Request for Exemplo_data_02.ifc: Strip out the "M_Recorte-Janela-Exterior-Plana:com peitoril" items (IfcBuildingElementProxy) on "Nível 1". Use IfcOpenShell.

First a look at what the model holds.

```python
import ifcopenshell
import ifcopenshell.util.element

model = ifcopenshell.open("Exemplo_data_02.ifc")
print(model.schema)
storey = next(s for s in model.by_type("IfcBuildingStorey") if s.Name == "Nível 1")
proxies = [e for e in ifcopenshell.util.element.get_decomposition(storey) if e.is_a("IfcBuildingElementProxy")]
seen = {}
for e in proxies:
    element_type = ifcopenshell.util.element.get_type(e)
    name = element_type.Name if element_type not in (None, e) else None
    seen[name] = seen.get(name, 0) + 1
for name, count in sorted(seen.items(), key=str):
    print(count, "x", name)
```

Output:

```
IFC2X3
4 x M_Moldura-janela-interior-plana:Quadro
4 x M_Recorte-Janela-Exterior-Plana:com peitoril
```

```python
import ifcopenshell
import ifcopenshell.api.root
import ifcopenshell.util.element

model = ifcopenshell.open("Exemplo_data_02.ifc")

storey = next(s for s in model.by_type("IfcBuildingStorey") if s.Name == "Nível 1")
proxies = [e for e in ifcopenshell.util.element.get_decomposition(storey) if e.is_a("IfcBuildingElementProxy")]
targets = [e for e in proxies if (t := ifcopenshell.util.element.get_type(e)) not in (None, e) and t.Name == "M_Recorte-Janela-Exterior-Plana:com peitoril"]

for e in targets:
    ifcopenshell.api.root.remove_product(model, product=e)
print(len(targets), "removed")

model.write("Exemplo_data_02_v2.ifc")
```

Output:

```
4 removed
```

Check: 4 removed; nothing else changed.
